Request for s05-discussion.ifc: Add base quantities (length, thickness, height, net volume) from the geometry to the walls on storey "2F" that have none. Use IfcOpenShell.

First a look at what the model holds.

```python
import ifcopenshell
import ifcopenshell.util.element
import ifcopenshell.util.unit

model = ifcopenshell.open("s05-discussion.ifc")
print(model.schema)
for unit_type in ("LENGTHUNIT", "AREAUNIT", "VOLUMEUNIT"):
    print(unit_type, ifcopenshell.util.unit.calculate_unit_scale(model, unit_type))
storey = next(s for s in model.by_type("IfcBuildingStorey") if s.Name == "2F")
walls = [e for e in ifcopenshell.util.element.get_decomposition(storey) if e.is_a("IfcWall")]
for e in sorted(walls, key=lambda e: e.id()):
    print(e.id(), e.is_a(), e.Name, list(ifcopenshell.util.element.get_psets(e, qtos_only=True)), sep=" | ")
```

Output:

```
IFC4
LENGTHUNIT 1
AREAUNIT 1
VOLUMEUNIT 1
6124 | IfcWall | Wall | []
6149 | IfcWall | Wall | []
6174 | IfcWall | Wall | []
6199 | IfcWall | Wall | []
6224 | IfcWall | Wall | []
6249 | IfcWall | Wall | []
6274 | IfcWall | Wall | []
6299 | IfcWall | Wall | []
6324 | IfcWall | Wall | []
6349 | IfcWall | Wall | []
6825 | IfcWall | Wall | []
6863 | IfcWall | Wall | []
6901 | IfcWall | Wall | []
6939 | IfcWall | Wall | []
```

```python
import ifcopenshell
import ifcopenshell.api.pset
import ifcopenshell.geom
import ifcopenshell.util.element
import ifcopenshell.util.shape
import ifcopenshell.util.unit

model = ifcopenshell.open("s05-discussion.ifc")
unit_scale = ifcopenshell.util.unit.calculate_unit_scale(model)
volume_scale = ifcopenshell.util.unit.calculate_unit_scale(model, "VOLUMEUNIT")
settings = ifcopenshell.geom.settings()

storey = next(s for s in model.by_type("IfcBuildingStorey") if s.Name == "2F")
walls = [e for e in ifcopenshell.util.element.get_decomposition(storey) if e.is_a("IfcWall")]

for e in sorted(walls, key=lambda e: e.id()):
    if ifcopenshell.util.element.get_psets(e, qtos_only=True, should_inherit=False):
        continue
    # Geometry comes back in metres, in the element's own axes.
    shape = ifcopenshell.geom.create_shape(settings, e)
    values = {
        "Length": ifcopenshell.util.shape.get_x(shape.geometry) / unit_scale,
        "Width": ifcopenshell.util.shape.get_y(shape.geometry) / unit_scale,
        "Height": ifcopenshell.util.shape.get_z(shape.geometry) / unit_scale,
        "NetVolume": ifcopenshell.util.shape.get_volume(shape.geometry) / volume_scale,
    }
    qto = ifcopenshell.api.pset.add_qto(model, product=e, name="Qto_WallBaseQuantities")
    ifcopenshell.api.pset.edit_qto(model, qto=qto, properties=values)
    print(e.id(), {k: round(v, 3) for k, v in values.items()})

model.write("s05-discussion-out.ifc")
```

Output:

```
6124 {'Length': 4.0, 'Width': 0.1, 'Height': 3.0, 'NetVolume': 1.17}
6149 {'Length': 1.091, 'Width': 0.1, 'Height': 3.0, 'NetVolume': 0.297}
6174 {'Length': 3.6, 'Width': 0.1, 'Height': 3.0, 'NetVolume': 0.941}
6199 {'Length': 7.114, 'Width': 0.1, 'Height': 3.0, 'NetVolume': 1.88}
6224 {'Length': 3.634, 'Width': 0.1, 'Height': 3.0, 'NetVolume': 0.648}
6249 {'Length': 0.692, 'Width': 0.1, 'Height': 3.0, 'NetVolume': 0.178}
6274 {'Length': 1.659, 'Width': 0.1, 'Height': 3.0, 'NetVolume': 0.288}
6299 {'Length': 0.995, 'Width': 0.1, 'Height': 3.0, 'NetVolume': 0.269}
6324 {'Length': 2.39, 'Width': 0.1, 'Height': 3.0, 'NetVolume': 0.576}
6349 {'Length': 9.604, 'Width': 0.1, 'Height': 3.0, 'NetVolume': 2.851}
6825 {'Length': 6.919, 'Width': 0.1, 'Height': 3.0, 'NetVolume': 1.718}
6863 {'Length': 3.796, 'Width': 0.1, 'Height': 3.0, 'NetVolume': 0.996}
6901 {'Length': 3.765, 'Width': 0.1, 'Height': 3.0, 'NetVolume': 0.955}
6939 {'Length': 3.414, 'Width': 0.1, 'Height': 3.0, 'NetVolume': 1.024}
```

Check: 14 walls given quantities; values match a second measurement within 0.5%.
